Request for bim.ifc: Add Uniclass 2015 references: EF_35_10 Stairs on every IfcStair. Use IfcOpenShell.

First a look at what the model holds.

```python
import ifcopenshell

model = ifcopenshell.open("bim.ifc")
print(model.schema)
print("classifications:", [c.Name for c in model.by_type("IfcClassification")])
for ifc_class in ("IfcDoor", "IfcRoof", "IfcStair", "IfcWall", "IfcWindow"):
    print(ifc_class, len(model.by_type(ifc_class)))
```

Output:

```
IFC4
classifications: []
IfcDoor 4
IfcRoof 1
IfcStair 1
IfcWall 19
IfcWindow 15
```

```python
import ifcopenshell
import ifcopenshell.api.classification

model = ifcopenshell.open("bim.ifc")

system = ifcopenshell.api.classification.add_classification(model, classification="Uniclass 2015")

codes = {
    "IfcStair": ("EF_35_10", "Stairs"),
}
for ifc_class, (code, name) in codes.items():
    products = model.by_type(ifc_class)
    ifcopenshell.api.classification.add_reference(
        model, products=products, classification=system, identification=code, name=name
    )
    print(code, len(products))

model.write("bim_edited.ifc")
```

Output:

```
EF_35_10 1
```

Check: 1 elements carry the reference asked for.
